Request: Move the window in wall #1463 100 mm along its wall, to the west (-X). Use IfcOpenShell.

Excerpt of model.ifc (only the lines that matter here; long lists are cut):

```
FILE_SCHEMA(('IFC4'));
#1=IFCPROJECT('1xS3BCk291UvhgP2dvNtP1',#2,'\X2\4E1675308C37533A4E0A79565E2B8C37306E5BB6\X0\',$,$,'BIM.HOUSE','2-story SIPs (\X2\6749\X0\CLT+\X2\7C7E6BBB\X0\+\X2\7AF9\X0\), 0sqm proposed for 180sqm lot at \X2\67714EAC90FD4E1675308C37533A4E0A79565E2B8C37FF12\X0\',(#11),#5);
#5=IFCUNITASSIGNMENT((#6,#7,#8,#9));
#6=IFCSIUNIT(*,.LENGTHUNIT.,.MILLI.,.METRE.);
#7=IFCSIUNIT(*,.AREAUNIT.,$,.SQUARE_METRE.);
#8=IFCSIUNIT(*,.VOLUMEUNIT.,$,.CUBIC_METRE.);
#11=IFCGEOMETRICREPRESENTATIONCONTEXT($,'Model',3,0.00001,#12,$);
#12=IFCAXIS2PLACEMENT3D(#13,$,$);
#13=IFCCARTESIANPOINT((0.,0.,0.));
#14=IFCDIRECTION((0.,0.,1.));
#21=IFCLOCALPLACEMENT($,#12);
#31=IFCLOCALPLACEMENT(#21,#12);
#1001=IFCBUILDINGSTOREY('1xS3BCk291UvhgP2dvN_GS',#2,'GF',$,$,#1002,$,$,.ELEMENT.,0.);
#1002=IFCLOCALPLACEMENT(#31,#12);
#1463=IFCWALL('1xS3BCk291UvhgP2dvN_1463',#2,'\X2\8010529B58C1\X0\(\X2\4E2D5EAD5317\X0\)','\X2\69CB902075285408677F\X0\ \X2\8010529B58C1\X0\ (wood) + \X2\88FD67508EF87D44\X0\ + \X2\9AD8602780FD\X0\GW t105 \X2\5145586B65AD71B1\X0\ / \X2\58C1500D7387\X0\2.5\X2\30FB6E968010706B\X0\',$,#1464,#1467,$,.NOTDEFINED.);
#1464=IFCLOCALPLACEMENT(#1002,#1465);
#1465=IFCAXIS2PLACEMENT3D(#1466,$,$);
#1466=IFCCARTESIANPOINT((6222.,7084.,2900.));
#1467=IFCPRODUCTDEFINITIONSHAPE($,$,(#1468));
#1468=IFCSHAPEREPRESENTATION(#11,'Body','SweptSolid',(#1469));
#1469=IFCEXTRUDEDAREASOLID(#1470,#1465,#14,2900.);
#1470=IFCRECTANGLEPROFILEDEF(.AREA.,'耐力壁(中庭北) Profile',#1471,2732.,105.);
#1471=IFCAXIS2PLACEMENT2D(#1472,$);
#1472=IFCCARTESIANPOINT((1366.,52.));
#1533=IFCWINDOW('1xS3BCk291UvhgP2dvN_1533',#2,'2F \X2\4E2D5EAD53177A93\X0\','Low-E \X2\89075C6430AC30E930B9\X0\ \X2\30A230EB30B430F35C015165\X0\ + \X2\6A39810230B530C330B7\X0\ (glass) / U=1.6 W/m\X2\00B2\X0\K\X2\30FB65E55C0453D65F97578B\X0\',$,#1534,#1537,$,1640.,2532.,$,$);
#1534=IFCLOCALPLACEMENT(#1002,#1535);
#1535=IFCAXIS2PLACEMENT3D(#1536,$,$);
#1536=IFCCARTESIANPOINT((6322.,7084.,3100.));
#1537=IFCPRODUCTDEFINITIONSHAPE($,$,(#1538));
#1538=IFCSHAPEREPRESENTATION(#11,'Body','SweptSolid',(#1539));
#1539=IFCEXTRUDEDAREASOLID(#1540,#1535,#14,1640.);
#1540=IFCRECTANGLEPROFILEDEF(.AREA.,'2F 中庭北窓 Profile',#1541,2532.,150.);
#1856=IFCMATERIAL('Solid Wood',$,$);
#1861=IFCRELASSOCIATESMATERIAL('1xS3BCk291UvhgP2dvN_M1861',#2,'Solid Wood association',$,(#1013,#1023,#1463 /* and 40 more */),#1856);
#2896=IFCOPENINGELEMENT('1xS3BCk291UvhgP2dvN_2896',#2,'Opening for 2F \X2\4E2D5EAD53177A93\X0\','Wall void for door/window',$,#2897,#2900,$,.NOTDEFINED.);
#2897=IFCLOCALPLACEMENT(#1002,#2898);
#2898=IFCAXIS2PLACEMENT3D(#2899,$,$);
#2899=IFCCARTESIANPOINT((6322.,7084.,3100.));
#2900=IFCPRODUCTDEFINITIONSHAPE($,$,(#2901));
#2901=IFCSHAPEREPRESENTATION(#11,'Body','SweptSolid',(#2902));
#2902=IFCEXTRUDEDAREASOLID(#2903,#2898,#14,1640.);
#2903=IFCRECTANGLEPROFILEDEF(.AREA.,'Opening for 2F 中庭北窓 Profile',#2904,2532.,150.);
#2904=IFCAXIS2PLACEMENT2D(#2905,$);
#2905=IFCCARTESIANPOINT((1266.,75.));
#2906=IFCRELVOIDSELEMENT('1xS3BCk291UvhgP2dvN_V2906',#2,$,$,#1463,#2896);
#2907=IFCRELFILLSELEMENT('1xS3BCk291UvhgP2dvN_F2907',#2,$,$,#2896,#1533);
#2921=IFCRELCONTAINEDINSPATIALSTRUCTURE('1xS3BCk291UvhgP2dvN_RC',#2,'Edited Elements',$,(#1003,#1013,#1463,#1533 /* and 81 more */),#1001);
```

```python
import ifcopenshell
import ifcopenshell.api.geometry
import ifcopenshell.util.placement
import ifcopenshell.util.unit

model = ifcopenshell.open("model.ifc")
unit_scale = ifcopenshell.util.unit.calculate_unit_scale(model)

window = model.by_guid("1xS3BCk291UvhgP2dvN_1533")
opening = window.FillsVoids[0].RelatingOpeningElement
wall = opening.VoidsElements[0].RelatingBuildingElement

wall_matrix = ifcopenshell.util.placement.get_local_placement(wall.ObjectPlacement)
shift = wall_matrix[:3, 0] * -0.1 / unit_scale
before = ifcopenshell.util.placement.get_local_placement(window.ObjectPlacement)[:3, 3].copy()

# The window is not placed relative to its opening, so move both.
for product in (opening, window):
    matrix = ifcopenshell.util.placement.get_local_placement(product.ObjectPlacement)
    matrix[:3, 3] += shift
    ifcopenshell.api.geometry.edit_object_placement(model, product=product, matrix=matrix, is_si=False)

after = ifcopenshell.util.placement.get_local_placement(window.ObjectPlacement)[:3, 3]
print("window moved by", (after - before).round(3) + 0.0)

model.write("model_updated.ifc")
```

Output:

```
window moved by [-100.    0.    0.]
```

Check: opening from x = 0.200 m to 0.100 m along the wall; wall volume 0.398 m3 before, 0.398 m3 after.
